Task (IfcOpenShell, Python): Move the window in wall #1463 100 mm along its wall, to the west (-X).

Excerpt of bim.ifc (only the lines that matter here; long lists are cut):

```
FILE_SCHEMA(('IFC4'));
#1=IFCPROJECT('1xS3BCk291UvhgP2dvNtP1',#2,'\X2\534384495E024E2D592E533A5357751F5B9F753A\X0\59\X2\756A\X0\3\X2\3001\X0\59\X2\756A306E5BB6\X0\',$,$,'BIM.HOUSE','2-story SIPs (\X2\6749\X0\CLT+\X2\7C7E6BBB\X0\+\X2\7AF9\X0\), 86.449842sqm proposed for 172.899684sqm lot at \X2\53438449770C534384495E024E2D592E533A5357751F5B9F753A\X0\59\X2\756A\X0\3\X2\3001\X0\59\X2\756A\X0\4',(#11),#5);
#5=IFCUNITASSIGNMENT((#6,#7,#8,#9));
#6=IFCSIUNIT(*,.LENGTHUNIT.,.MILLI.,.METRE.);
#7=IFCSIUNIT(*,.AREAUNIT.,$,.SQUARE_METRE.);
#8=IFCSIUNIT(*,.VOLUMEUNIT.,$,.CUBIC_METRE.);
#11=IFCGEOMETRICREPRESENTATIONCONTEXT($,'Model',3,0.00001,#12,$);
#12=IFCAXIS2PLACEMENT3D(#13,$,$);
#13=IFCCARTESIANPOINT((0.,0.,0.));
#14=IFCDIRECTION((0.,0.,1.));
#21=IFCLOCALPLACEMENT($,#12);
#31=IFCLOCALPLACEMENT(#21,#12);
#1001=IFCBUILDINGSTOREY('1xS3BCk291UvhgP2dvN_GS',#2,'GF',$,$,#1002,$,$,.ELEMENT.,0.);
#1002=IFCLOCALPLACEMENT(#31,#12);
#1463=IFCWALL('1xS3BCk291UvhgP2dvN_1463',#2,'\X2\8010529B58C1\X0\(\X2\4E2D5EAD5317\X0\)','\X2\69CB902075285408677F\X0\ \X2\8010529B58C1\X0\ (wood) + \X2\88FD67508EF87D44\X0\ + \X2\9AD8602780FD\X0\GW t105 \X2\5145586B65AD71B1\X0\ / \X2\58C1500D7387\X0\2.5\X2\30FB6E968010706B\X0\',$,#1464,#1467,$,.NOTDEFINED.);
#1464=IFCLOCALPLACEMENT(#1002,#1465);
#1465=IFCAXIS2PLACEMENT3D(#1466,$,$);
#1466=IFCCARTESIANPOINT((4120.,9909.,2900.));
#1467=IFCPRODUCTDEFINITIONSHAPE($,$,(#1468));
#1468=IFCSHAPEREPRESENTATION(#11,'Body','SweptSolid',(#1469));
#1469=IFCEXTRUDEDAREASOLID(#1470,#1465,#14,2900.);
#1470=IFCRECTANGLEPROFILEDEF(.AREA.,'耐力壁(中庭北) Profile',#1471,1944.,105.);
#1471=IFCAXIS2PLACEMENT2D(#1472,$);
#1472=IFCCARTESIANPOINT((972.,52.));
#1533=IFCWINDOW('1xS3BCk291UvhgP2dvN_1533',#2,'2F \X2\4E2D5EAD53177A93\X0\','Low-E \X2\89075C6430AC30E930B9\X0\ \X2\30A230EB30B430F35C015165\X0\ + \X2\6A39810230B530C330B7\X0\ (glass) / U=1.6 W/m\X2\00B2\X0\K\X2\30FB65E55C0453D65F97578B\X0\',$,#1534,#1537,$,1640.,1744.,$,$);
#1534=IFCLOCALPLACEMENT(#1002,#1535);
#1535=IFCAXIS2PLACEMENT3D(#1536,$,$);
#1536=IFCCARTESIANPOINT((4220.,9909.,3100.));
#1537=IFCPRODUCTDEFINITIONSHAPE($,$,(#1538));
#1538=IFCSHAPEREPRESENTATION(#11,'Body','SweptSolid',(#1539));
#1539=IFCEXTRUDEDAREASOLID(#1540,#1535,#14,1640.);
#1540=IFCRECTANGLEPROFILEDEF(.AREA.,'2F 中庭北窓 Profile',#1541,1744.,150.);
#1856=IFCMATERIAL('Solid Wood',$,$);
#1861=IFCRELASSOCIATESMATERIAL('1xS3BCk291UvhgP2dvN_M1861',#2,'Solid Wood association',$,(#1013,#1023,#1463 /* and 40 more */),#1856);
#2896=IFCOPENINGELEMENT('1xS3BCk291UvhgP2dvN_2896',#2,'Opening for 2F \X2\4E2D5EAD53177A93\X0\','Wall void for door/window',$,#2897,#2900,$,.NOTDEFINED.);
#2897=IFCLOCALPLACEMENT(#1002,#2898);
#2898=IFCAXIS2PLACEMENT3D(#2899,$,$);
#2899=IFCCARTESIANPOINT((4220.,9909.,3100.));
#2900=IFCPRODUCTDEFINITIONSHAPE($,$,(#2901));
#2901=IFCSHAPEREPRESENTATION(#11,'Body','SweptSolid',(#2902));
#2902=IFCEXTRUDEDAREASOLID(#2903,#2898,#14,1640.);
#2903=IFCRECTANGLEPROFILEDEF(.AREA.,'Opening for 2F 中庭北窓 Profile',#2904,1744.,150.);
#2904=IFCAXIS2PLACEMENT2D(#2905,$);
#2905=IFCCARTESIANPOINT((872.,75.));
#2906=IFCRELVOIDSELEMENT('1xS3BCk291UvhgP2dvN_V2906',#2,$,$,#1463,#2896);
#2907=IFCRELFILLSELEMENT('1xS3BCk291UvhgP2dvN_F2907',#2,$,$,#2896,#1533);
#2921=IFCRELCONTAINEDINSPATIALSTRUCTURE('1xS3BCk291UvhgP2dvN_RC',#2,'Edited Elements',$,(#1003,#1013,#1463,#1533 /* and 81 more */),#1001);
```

```python
import ifcopenshell
import ifcopenshell.api.geometry
import ifcopenshell.util.placement
import ifcopenshell.util.unit

model = ifcopenshell.open("bim.ifc")
unit_scale = ifcopenshell.util.unit.calculate_unit_scale(model)

window = model.by_guid("1xS3BCk291UvhgP2dvN_1533")
opening = window.FillsVoids[0].RelatingOpeningElement
wall = opening.VoidsElements[0].RelatingBuildingElement

wall_matrix = ifcopenshell.util.placement.get_local_placement(wall.ObjectPlacement)
shift = wall_matrix[:3, 0] * -0.1 / unit_scale
before = ifcopenshell.util.placement.get_local_placement(window.ObjectPlacement)[:3, 3].copy()

# The window is not placed relative to its opening, so move both.
for product in (opening, window):
    matrix = ifcopenshell.util.placement.get_local_placement(product.ObjectPlacement)
    matrix[:3, 3] += shift
    ifcopenshell.api.geometry.edit_object_placement(model, product=product, matrix=matrix, is_si=False)

after = ifcopenshell.util.placement.get_local_placement(window.ObjectPlacement)[:3, 3]
print("window moved by", (after - before).round(3) + 0.0)

model.write("bim_edited.ifc")
```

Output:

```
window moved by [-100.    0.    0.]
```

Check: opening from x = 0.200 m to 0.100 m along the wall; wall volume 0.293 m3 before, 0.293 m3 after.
